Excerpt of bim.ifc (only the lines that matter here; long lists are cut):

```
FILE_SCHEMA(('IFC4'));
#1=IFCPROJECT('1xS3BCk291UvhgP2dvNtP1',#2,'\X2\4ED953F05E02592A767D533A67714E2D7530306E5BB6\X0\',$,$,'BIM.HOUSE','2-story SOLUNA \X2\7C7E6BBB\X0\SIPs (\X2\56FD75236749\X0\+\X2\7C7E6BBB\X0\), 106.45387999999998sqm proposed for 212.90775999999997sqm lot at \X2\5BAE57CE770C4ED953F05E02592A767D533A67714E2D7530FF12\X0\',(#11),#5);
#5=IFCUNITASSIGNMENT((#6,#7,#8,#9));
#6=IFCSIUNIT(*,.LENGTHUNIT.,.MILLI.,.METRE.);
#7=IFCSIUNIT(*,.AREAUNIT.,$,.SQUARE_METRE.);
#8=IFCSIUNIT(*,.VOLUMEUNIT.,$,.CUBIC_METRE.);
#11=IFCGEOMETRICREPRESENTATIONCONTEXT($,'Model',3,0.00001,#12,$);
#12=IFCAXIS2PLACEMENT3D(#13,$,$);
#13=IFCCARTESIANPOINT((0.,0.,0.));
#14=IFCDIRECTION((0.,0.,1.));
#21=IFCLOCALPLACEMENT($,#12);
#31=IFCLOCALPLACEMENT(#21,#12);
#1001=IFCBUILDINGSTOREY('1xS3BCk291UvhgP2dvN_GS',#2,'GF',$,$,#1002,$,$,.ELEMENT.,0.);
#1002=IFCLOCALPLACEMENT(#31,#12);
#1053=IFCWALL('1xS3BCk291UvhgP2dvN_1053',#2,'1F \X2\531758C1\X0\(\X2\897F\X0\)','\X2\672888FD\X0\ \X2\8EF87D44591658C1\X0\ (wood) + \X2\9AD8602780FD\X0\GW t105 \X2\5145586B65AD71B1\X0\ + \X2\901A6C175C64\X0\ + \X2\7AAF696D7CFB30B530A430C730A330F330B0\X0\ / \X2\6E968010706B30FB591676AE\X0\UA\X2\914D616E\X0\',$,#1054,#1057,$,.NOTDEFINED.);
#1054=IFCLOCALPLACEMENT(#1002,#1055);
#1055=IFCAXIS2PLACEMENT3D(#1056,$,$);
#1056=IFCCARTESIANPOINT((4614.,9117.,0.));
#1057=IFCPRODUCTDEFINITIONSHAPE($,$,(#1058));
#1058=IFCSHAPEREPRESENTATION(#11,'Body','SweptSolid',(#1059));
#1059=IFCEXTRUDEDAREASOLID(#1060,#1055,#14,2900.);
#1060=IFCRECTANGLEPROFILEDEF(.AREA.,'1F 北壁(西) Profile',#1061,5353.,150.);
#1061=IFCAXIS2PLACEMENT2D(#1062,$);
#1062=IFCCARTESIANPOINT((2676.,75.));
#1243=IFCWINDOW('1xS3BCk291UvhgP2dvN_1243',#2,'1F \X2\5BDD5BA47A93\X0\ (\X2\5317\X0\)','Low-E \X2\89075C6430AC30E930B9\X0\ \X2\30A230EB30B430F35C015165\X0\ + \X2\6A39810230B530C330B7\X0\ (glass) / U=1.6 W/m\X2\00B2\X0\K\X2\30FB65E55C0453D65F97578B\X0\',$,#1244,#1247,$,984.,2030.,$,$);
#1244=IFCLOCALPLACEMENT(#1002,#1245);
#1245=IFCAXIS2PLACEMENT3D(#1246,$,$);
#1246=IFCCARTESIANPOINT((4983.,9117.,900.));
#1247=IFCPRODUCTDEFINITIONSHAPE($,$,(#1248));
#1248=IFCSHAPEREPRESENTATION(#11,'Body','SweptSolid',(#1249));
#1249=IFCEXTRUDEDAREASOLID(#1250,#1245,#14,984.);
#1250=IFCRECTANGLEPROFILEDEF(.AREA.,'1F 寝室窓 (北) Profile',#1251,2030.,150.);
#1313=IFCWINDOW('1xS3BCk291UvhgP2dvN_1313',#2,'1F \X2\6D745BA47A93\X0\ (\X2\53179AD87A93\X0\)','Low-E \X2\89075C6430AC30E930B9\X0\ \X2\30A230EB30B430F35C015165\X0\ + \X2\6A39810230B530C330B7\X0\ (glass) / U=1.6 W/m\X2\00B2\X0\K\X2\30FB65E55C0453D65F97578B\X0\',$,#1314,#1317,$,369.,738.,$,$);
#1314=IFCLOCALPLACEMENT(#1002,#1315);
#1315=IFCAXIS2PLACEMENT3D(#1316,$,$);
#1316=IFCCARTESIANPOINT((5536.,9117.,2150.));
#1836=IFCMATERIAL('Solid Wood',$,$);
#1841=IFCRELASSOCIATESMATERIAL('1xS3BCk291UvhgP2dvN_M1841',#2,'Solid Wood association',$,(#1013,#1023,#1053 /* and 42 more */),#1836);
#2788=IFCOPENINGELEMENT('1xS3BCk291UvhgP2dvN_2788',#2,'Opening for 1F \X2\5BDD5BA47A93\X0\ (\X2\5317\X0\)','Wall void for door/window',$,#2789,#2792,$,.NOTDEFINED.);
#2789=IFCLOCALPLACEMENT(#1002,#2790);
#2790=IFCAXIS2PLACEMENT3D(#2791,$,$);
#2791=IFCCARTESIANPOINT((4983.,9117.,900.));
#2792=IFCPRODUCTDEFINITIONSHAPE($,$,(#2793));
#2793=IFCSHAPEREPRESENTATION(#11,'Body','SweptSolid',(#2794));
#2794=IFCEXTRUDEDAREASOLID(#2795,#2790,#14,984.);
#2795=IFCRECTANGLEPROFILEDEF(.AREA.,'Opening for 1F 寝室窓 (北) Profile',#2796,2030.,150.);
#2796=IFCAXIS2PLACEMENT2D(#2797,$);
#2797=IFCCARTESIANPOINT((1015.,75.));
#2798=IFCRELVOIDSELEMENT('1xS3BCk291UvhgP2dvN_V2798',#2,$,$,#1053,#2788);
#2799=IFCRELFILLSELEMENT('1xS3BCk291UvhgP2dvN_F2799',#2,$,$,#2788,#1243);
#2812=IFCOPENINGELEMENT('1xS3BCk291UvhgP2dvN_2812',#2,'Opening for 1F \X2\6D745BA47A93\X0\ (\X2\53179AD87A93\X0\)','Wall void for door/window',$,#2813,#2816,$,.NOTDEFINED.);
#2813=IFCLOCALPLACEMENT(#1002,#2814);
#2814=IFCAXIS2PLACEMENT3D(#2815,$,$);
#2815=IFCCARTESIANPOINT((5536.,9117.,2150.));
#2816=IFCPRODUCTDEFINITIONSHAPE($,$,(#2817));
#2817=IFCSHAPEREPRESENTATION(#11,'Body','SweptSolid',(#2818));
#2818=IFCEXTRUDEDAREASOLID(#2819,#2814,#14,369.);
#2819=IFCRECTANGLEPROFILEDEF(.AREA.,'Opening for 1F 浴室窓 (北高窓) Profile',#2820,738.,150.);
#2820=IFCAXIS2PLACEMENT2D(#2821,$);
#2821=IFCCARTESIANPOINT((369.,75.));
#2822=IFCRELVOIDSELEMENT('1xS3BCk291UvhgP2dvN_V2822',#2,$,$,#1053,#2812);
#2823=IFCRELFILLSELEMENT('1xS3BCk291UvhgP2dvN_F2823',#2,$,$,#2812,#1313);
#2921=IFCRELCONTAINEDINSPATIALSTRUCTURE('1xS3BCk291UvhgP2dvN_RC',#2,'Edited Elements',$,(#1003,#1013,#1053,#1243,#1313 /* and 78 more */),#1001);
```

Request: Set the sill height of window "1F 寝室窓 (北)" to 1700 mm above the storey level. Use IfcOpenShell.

```python
import numpy as np
import ifcopenshell
import ifcopenshell.api.geometry
import ifcopenshell.geom
import ifcopenshell.util.element
import ifcopenshell.util.placement
import ifcopenshell.util.shape
import ifcopenshell.util.unit

model = ifcopenshell.open("bim.ifc")
unit_scale = ifcopenshell.util.unit.calculate_unit_scale(model)

window = model.by_id(1243)
opening = window.FillsVoids[0].RelatingOpeningElement
storey = ifcopenshell.util.element.get_container(window, ifc_class="IfcBuildingStorey")
level = ifcopenshell.util.placement.get_local_placement(storey.ObjectPlacement)[2, 3]

# The opening's origin need not be at the sill, so measure its lowest point.
shape = ifcopenshell.geom.create_shape(ifcopenshell.geom.settings(), opening)
bottom = ifcopenshell.util.shape.get_shape_bottom_elevation(shape, shape.geometry) / unit_scale
dz = level + 1.7 / unit_scale - bottom

shift = np.array([0.0, 0.0, dz])
# The window is not placed relative to its opening, so move both.
for product in (opening, window):
    matrix = ifcopenshell.util.placement.get_local_placement(product.ObjectPlacement)
    matrix[:3, 3] += shift
    ifcopenshell.api.geometry.edit_object_placement(model, product=product, matrix=matrix, is_si=False)

print(f"moved by {dz * unit_scale:+.3f} m")

model.write("bim_edited.ifc")
```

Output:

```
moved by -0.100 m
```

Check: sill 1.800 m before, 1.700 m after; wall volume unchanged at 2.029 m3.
